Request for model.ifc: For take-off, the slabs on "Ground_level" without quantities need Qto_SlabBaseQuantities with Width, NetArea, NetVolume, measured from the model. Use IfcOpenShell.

First a look at what the model holds.

```python
import ifcopenshell
import ifcopenshell.util.element
import ifcopenshell.util.unit

model = ifcopenshell.open("model.ifc")
print(model.schema)
for unit_type in ("LENGTHUNIT", "AREAUNIT", "VOLUMEUNIT"):
    print(unit_type, ifcopenshell.util.unit.calculate_unit_scale(model, unit_type))
storey = next(s for s in model.by_type("IfcBuildingStorey") if s.Name == "Ground_level")
slabs = [e for e in ifcopenshell.util.element.get_decomposition(storey) if e.is_a("IfcSlab")]
for e in sorted(slabs, key=lambda e: e.id()):
    print(e.id(), e.is_a(), e.Name, list(ifcopenshell.util.element.get_psets(e, qtos_only=True)), sep=" | ")
```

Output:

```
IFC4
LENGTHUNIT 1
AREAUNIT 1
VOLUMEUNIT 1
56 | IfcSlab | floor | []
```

```python
import ifcopenshell
import ifcopenshell.api.pset
import ifcopenshell.geom
import ifcopenshell.util.element
import ifcopenshell.util.shape
import ifcopenshell.util.unit

model = ifcopenshell.open("model.ifc")
unit_scale = ifcopenshell.util.unit.calculate_unit_scale(model)
area_scale = ifcopenshell.util.unit.calculate_unit_scale(model, "AREAUNIT")
volume_scale = ifcopenshell.util.unit.calculate_unit_scale(model, "VOLUMEUNIT")
settings = ifcopenshell.geom.settings()

storey = next(s for s in model.by_type("IfcBuildingStorey") if s.Name == "Ground_level")
slabs = [e for e in ifcopenshell.util.element.get_decomposition(storey) if e.is_a("IfcSlab")]

for e in sorted(slabs, key=lambda e: e.id()):
    if ifcopenshell.util.element.get_psets(e, qtos_only=True, should_inherit=False):
        continue
    # Geometry comes back in metres, in the element's own axes.
    shape = ifcopenshell.geom.create_shape(settings, e)
    values = {
        "Width": ifcopenshell.util.shape.get_z(shape.geometry) / unit_scale,
        "NetArea": ifcopenshell.util.shape.get_footprint_area(shape.geometry) / area_scale,
        "NetVolume": ifcopenshell.util.shape.get_volume(shape.geometry) / volume_scale,
    }
    qto = ifcopenshell.api.pset.add_qto(model, product=e, name="Qto_SlabBaseQuantities")
    ifcopenshell.api.pset.edit_qto(model, qto=qto, properties=values)
    print(e.id(), {k: round(v, 3) for k, v in values.items()})

model.write("model-out.ifc")
```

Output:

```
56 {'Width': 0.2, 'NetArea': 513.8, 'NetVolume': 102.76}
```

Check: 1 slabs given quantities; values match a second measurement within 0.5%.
